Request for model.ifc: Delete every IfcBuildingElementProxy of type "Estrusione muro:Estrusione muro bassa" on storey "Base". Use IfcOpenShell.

First a look at what the model holds.

```python
import ifcopenshell
import ifcopenshell.util.element

model = ifcopenshell.open("model.ifc")
print(model.schema)
storey = next(s for s in model.by_type("IfcBuildingStorey") if s.Name == "Base")
proxies = [e for e in ifcopenshell.util.element.get_decomposition(storey) if e.is_a("IfcBuildingElementProxy")]
seen = {}
for e in proxies:
    element_type = ifcopenshell.util.element.get_type(e)
    name = element_type.Name if element_type not in (None, e) else None
    seen[name] = seen.get(name, 0) + 1
for name, count in sorted(seen.items(), key=str):
    print(count, "x", name)
```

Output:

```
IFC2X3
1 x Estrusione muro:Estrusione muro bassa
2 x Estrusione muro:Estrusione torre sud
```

```python
import ifcopenshell
import ifcopenshell.api.root
import ifcopenshell.util.element

model = ifcopenshell.open("model.ifc")

storey = next(s for s in model.by_type("IfcBuildingStorey") if s.Name == "Base")
proxies = [e for e in ifcopenshell.util.element.get_decomposition(storey) if e.is_a("IfcBuildingElementProxy")]
targets = [e for e in proxies if (t := ifcopenshell.util.element.get_type(e)) not in (None, e) and t.Name == "Estrusione muro:Estrusione muro bassa"]

for e in targets:
    ifcopenshell.api.root.remove_product(model, product=e)
print(len(targets), "removed")

model.write("model_edited.ifc")
```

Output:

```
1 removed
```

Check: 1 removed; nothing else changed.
